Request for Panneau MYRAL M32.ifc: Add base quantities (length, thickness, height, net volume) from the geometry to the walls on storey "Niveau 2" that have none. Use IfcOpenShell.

First a look at what the model holds.

```python
import ifcopenshell
import ifcopenshell.util.element
import ifcopenshell.util.unit

model = ifcopenshell.open("Panneau MYRAL M32.ifc")
print(model.schema)
for unit_type in ("LENGTHUNIT", "AREAUNIT", "VOLUMEUNIT"):
    print(unit_type, ifcopenshell.util.unit.calculate_unit_scale(model, unit_type))
storey = next(s for s in model.by_type("IfcBuildingStorey") if s.Name == "Niveau 2")
walls = [e for e in ifcopenshell.util.element.get_decomposition(storey) if e.is_a("IfcWall")]
for e in sorted(walls, key=lambda e: e.id()):
    print(e.id(), e.is_a(), e.Name, list(ifcopenshell.util.element.get_psets(e, qtos_only=True)), sep=" | ")
```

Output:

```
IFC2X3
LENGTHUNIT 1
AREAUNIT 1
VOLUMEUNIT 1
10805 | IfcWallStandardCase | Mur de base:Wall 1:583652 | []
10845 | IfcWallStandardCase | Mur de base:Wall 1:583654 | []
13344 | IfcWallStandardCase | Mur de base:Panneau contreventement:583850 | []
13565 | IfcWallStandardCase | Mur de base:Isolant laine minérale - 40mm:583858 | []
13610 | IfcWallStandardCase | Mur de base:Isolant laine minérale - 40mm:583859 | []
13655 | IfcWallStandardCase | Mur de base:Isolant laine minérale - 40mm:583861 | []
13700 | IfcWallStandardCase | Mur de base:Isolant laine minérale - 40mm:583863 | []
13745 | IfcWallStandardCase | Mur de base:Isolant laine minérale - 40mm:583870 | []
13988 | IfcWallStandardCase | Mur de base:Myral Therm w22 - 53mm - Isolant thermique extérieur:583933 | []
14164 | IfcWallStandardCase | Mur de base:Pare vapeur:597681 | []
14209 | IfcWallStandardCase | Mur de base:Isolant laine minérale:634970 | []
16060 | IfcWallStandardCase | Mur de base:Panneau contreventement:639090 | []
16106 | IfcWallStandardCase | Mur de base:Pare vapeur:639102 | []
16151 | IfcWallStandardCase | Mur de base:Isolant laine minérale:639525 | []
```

```python
import ifcopenshell
import ifcopenshell.api.pset
import ifcopenshell.geom
import ifcopenshell.util.element
import ifcopenshell.util.shape
import ifcopenshell.util.unit

model = ifcopenshell.open("Panneau MYRAL M32.ifc")
unit_scale = ifcopenshell.util.unit.calculate_unit_scale(model)
volume_scale = ifcopenshell.util.unit.calculate_unit_scale(model, "VOLUMEUNIT")
settings = ifcopenshell.geom.settings()

storey = next(s for s in model.by_type("IfcBuildingStorey") if s.Name == "Niveau 2")
walls = [e for e in ifcopenshell.util.element.get_decomposition(storey) if e.is_a("IfcWall")]

for e in sorted(walls, key=lambda e: e.id()):
    if ifcopenshell.util.element.get_psets(e, qtos_only=True, should_inherit=False):
        continue
    # Geometry comes back in metres, in the element's own axes.
    shape = ifcopenshell.geom.create_shape(settings, e)
    values = {
        "Length": ifcopenshell.util.shape.get_x(shape.geometry) / unit_scale,
        "Width": ifcopenshell.util.shape.get_y(shape.geometry) / unit_scale,
        "Height": ifcopenshell.util.shape.get_z(shape.geometry) / unit_scale,
        "NetVolume": ifcopenshell.util.shape.get_volume(shape.geometry) / volume_scale,
    }
    qto = ifcopenshell.api.pset.add_qto(model, product=e, name="BaseQuantities")
    ifcopenshell.api.pset.edit_qto(model, qto=qto, properties=values)
    print(e.id(), {k: round(v, 3) for k, v in values.items()})

model.write("Panneau MYRAL M32_v2.ifc")
```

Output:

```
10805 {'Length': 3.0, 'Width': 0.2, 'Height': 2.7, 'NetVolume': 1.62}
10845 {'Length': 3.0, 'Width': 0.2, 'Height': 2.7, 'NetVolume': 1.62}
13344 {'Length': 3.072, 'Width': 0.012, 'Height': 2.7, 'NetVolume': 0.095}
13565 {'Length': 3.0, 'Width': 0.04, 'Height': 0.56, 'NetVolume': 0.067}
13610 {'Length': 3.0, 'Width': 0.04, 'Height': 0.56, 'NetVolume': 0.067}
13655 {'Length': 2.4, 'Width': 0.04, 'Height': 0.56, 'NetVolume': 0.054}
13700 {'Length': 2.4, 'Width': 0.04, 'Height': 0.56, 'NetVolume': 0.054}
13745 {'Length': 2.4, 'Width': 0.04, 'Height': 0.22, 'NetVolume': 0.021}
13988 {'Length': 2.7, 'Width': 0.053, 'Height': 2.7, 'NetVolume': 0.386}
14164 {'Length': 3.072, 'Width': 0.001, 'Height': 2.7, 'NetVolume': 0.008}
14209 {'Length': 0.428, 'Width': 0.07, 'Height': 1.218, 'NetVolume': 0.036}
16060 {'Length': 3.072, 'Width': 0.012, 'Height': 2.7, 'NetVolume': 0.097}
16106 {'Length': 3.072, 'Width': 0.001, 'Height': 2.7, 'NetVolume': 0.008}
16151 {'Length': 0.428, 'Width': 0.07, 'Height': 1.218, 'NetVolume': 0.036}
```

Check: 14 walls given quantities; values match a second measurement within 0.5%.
